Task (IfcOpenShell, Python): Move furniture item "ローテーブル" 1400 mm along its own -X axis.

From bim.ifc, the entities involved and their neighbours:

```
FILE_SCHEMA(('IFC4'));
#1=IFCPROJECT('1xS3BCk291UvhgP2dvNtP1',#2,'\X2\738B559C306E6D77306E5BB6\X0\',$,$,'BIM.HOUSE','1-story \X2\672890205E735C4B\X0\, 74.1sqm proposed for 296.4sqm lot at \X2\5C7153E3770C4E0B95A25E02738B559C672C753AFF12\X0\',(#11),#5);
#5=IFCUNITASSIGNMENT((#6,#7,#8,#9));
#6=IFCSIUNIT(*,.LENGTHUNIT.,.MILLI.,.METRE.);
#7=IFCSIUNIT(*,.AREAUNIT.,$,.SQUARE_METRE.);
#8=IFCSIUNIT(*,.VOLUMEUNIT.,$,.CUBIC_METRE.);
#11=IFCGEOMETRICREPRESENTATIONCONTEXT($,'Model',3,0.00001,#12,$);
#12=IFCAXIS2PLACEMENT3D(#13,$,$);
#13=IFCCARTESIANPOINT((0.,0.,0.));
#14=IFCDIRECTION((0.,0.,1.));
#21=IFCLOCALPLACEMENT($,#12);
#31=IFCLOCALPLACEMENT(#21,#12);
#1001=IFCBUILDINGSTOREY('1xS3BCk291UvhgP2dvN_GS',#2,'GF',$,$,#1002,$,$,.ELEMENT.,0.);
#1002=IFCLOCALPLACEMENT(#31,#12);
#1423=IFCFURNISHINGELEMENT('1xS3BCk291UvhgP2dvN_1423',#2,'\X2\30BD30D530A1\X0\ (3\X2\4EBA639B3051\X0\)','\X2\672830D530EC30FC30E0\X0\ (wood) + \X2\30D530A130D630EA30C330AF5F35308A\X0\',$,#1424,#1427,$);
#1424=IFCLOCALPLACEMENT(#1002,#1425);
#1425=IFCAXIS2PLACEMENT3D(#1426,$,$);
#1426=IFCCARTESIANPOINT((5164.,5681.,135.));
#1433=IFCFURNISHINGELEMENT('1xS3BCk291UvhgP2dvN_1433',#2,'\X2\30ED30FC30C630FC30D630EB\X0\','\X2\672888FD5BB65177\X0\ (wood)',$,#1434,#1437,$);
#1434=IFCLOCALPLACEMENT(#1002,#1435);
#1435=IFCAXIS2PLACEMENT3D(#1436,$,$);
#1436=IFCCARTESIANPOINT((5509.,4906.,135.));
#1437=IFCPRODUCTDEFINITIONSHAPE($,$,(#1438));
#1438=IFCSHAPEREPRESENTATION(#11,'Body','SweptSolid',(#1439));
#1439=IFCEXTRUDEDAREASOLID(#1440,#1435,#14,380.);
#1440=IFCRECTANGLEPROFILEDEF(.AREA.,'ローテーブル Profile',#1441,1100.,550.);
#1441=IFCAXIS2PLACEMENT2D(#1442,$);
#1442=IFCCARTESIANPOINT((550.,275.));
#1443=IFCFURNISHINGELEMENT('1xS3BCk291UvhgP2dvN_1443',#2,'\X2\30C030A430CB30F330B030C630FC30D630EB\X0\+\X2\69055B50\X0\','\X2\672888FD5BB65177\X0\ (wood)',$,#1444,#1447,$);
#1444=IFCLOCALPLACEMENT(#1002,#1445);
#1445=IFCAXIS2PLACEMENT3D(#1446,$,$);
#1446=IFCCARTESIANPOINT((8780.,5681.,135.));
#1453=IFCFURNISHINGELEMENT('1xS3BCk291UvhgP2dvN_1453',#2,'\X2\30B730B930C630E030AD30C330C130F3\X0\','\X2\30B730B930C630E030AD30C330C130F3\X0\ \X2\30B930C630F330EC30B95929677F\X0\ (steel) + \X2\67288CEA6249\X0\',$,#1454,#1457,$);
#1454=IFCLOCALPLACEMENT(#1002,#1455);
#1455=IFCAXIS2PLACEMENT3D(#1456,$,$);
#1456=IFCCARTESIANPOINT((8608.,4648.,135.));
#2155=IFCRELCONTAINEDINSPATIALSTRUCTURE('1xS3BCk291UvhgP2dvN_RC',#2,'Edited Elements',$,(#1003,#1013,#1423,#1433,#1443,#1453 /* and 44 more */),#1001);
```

```python
import ifcopenshell
import ifcopenshell.api.geometry
import ifcopenshell.util.placement
import ifcopenshell.util.unit

model = ifcopenshell.open("bim.ifc")
unit_scale = ifcopenshell.util.unit.calculate_unit_scale(model)

item = model.by_id(1433)
matrix = ifcopenshell.util.placement.get_local_placement(item.ObjectPlacement)
matrix[:3, 3] -= matrix[:3, 0] * 1.4 / unit_scale
ifcopenshell.api.geometry.edit_object_placement(model, product=item, matrix=matrix, is_si=False)

print(ifcopenshell.util.placement.get_local_placement(item.ObjectPlacement).round(3) + 0.0)

model.write("bim_v2.ifc")
```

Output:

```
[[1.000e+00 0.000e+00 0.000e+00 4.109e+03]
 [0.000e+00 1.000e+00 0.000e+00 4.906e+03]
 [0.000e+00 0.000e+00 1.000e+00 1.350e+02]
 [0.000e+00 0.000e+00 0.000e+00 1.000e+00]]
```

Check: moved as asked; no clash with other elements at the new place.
